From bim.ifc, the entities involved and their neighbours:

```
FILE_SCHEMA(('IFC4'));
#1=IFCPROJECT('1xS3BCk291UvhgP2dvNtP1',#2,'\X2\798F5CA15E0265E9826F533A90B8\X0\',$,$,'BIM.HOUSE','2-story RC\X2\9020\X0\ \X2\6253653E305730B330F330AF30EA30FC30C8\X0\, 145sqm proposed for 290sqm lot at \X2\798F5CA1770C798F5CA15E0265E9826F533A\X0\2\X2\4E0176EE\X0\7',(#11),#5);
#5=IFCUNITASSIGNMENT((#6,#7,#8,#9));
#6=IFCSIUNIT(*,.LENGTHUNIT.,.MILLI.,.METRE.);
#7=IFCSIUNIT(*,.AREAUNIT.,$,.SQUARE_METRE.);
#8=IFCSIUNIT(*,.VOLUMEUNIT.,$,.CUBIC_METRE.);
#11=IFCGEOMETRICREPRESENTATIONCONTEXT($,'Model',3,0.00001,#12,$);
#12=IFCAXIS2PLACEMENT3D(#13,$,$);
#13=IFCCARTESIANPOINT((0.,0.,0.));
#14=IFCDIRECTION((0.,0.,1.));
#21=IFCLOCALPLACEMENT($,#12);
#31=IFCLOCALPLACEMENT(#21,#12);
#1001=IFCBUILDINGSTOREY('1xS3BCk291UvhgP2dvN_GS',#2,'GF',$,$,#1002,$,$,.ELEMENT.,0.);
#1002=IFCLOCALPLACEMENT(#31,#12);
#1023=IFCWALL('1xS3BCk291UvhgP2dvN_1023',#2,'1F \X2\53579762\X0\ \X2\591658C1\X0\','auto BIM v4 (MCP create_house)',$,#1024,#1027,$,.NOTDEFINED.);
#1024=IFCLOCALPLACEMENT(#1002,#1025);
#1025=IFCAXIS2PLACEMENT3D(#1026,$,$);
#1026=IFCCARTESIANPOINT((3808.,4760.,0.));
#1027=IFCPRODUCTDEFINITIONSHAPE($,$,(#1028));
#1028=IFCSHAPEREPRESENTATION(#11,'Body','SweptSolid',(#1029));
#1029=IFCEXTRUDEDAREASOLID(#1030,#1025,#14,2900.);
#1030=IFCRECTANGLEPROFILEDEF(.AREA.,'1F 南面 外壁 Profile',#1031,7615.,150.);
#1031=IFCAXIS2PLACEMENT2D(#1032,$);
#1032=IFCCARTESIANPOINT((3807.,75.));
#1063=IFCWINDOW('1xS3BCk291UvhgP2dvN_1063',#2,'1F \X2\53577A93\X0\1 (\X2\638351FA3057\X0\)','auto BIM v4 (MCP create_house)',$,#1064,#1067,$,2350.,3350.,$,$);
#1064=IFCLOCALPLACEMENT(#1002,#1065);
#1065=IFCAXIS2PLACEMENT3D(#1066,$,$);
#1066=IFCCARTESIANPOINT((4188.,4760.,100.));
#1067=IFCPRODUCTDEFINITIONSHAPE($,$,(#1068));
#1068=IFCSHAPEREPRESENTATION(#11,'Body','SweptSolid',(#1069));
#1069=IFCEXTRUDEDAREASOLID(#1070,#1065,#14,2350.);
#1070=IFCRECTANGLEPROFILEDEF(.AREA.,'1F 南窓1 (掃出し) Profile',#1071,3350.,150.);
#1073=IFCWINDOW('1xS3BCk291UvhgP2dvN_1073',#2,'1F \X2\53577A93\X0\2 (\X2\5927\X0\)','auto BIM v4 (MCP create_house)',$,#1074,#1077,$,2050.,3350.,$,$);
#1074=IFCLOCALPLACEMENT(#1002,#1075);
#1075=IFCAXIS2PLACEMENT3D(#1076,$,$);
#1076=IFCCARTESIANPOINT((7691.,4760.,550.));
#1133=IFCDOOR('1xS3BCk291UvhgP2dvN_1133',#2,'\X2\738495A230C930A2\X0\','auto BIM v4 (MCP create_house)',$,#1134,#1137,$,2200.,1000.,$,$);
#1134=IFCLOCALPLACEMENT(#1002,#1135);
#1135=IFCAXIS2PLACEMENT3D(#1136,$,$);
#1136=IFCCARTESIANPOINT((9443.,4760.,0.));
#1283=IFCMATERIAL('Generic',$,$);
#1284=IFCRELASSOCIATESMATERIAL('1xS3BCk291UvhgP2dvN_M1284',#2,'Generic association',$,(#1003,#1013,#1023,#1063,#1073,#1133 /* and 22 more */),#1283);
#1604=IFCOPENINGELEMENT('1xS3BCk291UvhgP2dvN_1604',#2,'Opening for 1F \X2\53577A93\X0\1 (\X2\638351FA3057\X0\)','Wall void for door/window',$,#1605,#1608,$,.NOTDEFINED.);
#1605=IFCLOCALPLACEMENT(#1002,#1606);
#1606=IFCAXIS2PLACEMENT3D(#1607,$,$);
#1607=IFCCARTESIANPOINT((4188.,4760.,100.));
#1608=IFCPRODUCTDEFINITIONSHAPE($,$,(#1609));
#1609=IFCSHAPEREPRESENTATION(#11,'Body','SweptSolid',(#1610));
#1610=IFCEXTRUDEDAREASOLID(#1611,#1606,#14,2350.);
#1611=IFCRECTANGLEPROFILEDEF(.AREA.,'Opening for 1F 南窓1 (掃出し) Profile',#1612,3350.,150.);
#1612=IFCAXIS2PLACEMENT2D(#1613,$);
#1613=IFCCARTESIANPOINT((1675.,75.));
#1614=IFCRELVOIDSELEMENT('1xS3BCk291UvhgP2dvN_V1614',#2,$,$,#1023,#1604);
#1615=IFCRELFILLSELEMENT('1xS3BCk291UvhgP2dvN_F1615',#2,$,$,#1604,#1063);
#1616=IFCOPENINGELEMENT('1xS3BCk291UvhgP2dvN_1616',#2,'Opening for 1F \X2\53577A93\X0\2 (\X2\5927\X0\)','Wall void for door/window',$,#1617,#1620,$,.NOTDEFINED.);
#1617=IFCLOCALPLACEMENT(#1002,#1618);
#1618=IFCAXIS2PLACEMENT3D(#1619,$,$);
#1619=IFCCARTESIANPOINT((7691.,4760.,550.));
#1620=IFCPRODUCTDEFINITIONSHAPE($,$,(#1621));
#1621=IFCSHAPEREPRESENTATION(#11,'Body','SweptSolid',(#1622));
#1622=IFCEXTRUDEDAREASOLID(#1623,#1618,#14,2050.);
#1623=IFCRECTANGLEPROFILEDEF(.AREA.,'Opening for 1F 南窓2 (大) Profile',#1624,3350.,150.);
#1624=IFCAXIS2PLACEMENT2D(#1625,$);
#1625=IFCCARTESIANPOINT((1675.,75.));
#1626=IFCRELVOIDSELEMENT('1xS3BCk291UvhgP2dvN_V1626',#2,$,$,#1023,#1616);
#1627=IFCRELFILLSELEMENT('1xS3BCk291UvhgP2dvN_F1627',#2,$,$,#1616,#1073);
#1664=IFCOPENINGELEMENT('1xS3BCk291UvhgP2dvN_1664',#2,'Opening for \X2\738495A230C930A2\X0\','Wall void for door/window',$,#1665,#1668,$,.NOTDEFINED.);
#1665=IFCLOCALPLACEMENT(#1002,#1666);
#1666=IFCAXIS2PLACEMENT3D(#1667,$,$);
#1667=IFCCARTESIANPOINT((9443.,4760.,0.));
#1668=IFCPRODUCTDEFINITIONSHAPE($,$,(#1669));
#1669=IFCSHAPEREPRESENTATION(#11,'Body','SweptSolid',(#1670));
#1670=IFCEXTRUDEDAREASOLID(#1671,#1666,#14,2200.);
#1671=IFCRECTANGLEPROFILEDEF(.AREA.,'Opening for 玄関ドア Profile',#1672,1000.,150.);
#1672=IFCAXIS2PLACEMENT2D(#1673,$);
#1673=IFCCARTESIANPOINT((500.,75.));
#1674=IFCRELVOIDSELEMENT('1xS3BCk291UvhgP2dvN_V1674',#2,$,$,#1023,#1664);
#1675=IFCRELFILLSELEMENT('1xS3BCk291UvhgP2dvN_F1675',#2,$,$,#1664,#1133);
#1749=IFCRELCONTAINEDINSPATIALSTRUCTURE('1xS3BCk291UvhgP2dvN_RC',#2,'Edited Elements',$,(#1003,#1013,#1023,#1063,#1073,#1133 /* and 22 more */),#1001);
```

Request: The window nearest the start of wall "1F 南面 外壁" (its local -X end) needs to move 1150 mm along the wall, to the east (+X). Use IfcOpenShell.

```python
import ifcopenshell
import ifcopenshell.api.geometry
import ifcopenshell.util.placement

model = ifcopenshell.open("bim.ifc")

window = model.by_guid("1xS3BCk291UvhgP2dvN_1063")
opening = window.FillsVoids[0].RelatingOpeningElement
wall = opening.VoidsElements[0].RelatingBuildingElement

wall_matrix = ifcopenshell.util.placement.get_local_placement(wall.ObjectPlacement)
shift = wall_matrix[:3, 0] * 1150.0
before = ifcopenshell.util.placement.get_local_placement(window.ObjectPlacement)[:3, 3].copy()

# The window is not placed relative to its opening, so move both.
for product in (opening, window):
    matrix = ifcopenshell.util.placement.get_local_placement(product.ObjectPlacement)
    matrix[:3, 3] += shift
    ifcopenshell.api.geometry.edit_object_placement(model, product=product, matrix=matrix, is_si=False)

after = ifcopenshell.util.placement.get_local_placement(window.ObjectPlacement)[:3, 3]
print("window moved by", (after - before).round(3) + 0.0)

model.write("bim_edited.ifc")
```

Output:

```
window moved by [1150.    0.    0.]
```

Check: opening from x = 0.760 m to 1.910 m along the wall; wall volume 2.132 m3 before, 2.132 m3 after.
